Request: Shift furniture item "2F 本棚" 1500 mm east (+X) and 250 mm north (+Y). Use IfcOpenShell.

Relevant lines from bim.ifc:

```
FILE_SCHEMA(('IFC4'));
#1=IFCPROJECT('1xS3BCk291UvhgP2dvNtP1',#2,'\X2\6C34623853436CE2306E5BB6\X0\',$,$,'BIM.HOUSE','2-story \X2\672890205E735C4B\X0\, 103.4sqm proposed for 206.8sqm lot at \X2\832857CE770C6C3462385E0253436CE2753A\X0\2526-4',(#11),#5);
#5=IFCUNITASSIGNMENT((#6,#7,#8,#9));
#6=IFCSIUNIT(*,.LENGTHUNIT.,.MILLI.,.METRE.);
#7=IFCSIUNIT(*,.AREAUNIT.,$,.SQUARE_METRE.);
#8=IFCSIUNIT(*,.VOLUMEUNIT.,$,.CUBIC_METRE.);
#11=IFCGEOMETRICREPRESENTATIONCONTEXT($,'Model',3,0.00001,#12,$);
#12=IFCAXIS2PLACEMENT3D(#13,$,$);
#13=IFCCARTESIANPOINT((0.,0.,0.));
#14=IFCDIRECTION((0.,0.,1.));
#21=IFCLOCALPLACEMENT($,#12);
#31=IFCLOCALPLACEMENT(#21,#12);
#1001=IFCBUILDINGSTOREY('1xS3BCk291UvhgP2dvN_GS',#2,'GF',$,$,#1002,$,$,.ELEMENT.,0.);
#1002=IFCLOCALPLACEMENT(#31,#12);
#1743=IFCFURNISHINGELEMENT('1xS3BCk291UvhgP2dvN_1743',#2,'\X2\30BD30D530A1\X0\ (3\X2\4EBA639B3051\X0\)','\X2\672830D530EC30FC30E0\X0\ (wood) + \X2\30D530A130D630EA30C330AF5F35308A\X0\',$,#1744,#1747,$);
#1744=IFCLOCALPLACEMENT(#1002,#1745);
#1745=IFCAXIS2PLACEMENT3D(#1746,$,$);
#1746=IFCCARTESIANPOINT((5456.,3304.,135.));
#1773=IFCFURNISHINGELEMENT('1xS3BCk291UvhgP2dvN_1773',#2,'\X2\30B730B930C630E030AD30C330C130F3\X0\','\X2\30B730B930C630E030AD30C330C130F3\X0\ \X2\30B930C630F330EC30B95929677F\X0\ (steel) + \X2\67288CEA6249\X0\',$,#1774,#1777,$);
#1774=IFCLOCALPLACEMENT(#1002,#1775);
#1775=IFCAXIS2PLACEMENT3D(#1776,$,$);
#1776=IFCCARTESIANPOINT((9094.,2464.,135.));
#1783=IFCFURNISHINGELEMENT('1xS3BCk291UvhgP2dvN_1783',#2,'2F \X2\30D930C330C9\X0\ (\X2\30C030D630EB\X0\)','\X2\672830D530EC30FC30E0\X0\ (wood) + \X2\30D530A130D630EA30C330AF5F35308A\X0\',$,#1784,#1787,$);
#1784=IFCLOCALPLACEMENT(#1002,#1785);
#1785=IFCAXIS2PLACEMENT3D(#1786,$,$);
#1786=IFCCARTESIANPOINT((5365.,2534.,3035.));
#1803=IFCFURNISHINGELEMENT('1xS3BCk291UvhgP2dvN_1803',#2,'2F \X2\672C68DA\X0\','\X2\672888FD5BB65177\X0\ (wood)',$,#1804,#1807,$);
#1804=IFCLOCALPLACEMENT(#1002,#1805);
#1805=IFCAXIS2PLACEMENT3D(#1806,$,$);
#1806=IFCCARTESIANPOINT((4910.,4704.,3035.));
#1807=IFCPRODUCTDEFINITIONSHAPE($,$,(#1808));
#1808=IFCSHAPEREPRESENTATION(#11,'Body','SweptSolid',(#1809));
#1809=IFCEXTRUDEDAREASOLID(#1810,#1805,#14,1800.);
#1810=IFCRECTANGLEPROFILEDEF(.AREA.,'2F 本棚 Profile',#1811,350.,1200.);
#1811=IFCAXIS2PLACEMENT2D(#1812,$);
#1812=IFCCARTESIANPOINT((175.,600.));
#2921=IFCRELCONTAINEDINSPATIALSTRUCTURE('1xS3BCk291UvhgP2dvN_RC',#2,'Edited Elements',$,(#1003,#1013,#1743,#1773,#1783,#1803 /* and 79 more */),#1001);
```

```python
import ifcopenshell
import ifcopenshell.api.geometry
import ifcopenshell.util.placement

model = ifcopenshell.open("bim.ifc")

item = model.by_id(1803)
matrix = ifcopenshell.util.placement.get_local_placement(item.ObjectPlacement)
matrix[0, 3] += 1500.0
matrix[1, 3] += 250.0
ifcopenshell.api.geometry.edit_object_placement(model, product=item, matrix=matrix, is_si=False)

print(ifcopenshell.util.placement.get_local_placement(item.ObjectPlacement).round(3) + 0.0)

model.write("bim_edited.ifc")
```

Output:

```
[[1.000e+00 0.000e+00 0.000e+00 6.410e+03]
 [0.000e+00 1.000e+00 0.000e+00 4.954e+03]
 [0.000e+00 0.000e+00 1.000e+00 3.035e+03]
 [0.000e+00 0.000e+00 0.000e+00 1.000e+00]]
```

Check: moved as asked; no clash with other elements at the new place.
